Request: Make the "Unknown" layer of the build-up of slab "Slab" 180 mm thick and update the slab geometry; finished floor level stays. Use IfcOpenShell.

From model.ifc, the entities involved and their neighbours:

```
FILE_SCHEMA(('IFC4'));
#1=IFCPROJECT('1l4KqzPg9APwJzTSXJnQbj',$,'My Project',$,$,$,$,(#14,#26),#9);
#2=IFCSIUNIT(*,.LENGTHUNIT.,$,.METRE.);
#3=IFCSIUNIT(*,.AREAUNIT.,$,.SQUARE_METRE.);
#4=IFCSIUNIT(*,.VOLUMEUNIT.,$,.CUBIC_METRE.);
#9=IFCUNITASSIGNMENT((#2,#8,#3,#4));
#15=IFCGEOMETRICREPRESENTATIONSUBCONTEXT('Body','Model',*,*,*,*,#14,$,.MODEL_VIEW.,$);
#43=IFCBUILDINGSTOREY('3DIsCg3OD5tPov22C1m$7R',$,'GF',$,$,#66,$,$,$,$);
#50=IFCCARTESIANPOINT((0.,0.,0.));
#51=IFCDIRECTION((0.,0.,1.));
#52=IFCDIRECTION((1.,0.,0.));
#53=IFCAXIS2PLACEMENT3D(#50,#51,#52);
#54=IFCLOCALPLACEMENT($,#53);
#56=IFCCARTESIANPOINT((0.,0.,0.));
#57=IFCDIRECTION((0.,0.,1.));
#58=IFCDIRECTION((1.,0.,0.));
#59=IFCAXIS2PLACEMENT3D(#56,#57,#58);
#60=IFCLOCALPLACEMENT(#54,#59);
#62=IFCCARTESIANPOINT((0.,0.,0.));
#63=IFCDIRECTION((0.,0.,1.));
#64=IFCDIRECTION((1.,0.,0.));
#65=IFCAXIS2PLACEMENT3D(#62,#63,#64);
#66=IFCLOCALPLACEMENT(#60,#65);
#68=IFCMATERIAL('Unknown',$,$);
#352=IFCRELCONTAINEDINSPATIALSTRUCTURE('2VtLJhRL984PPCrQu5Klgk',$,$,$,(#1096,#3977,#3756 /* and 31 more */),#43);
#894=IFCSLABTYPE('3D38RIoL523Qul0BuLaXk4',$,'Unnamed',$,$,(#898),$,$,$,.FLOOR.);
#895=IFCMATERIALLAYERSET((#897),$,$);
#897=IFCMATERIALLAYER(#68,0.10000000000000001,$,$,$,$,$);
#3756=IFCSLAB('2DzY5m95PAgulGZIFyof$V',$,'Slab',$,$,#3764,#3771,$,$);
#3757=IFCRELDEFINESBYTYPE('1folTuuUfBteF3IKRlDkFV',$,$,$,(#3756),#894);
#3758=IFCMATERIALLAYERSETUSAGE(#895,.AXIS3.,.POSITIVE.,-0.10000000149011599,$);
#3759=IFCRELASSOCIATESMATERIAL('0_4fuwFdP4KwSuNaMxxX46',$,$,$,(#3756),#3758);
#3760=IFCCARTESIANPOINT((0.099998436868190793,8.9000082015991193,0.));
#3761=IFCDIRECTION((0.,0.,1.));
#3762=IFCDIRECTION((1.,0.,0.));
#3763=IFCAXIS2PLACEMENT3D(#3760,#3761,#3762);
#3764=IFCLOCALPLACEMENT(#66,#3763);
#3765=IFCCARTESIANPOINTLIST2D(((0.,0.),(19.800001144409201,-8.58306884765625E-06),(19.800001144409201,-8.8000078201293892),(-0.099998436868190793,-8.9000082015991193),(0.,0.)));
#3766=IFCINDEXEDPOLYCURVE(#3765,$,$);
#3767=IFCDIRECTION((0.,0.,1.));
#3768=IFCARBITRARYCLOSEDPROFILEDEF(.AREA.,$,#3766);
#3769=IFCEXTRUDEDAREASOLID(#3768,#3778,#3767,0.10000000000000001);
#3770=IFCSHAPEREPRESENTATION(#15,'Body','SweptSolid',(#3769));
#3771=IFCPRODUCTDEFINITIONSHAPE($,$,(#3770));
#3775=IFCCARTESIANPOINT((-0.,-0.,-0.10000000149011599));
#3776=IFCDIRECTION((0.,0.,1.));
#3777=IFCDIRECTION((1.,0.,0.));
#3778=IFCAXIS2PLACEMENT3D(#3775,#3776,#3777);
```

```python
import ifcopenshell
import ifcopenshell.util.element
import ifcopenshell.util.representation

model = ifcopenshell.open("model.ifc")

layer_set = model.by_id(895)
layer = next(l for l in layer_set.MaterialLayers if l.Material and l.Material.Name == "Unknown")
change = 0.18 - layer.LayerThickness
layer.LayerThickness += change

# Geometry does not follow the layer set by itself.
slabs = [e for e in ifcopenshell.util.element.get_elements_by_material(model, layer_set) if e.is_a("IfcSlab")]
for slab in sorted(slabs, key=lambda e: e.id()):
    body = ifcopenshell.util.representation.get_representation(slab, "Model", "Body")
    solid = body.Items[0]
    old_depth = solid.Depth
    solid.Depth += change
    # Extruded upwards: lower the start of the extrusion so the top stays.
    x, y, z = solid.Position.Location.Coordinates
    solid.Position.Location = model.createIfcCartesianPoint((x, y, z - change))
    print(slab.id(), f"{old_depth:g} -> {solid.Depth:g}")

# The layers are counted up from the underside, which has moved.
for usage in {ifcopenshell.util.element.get_material(slab) for slab in slabs}:
    usage.OffsetFromReferenceLine -= change

model.write("model_v2.ifc")
```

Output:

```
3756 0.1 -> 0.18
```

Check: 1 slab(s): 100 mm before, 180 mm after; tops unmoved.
